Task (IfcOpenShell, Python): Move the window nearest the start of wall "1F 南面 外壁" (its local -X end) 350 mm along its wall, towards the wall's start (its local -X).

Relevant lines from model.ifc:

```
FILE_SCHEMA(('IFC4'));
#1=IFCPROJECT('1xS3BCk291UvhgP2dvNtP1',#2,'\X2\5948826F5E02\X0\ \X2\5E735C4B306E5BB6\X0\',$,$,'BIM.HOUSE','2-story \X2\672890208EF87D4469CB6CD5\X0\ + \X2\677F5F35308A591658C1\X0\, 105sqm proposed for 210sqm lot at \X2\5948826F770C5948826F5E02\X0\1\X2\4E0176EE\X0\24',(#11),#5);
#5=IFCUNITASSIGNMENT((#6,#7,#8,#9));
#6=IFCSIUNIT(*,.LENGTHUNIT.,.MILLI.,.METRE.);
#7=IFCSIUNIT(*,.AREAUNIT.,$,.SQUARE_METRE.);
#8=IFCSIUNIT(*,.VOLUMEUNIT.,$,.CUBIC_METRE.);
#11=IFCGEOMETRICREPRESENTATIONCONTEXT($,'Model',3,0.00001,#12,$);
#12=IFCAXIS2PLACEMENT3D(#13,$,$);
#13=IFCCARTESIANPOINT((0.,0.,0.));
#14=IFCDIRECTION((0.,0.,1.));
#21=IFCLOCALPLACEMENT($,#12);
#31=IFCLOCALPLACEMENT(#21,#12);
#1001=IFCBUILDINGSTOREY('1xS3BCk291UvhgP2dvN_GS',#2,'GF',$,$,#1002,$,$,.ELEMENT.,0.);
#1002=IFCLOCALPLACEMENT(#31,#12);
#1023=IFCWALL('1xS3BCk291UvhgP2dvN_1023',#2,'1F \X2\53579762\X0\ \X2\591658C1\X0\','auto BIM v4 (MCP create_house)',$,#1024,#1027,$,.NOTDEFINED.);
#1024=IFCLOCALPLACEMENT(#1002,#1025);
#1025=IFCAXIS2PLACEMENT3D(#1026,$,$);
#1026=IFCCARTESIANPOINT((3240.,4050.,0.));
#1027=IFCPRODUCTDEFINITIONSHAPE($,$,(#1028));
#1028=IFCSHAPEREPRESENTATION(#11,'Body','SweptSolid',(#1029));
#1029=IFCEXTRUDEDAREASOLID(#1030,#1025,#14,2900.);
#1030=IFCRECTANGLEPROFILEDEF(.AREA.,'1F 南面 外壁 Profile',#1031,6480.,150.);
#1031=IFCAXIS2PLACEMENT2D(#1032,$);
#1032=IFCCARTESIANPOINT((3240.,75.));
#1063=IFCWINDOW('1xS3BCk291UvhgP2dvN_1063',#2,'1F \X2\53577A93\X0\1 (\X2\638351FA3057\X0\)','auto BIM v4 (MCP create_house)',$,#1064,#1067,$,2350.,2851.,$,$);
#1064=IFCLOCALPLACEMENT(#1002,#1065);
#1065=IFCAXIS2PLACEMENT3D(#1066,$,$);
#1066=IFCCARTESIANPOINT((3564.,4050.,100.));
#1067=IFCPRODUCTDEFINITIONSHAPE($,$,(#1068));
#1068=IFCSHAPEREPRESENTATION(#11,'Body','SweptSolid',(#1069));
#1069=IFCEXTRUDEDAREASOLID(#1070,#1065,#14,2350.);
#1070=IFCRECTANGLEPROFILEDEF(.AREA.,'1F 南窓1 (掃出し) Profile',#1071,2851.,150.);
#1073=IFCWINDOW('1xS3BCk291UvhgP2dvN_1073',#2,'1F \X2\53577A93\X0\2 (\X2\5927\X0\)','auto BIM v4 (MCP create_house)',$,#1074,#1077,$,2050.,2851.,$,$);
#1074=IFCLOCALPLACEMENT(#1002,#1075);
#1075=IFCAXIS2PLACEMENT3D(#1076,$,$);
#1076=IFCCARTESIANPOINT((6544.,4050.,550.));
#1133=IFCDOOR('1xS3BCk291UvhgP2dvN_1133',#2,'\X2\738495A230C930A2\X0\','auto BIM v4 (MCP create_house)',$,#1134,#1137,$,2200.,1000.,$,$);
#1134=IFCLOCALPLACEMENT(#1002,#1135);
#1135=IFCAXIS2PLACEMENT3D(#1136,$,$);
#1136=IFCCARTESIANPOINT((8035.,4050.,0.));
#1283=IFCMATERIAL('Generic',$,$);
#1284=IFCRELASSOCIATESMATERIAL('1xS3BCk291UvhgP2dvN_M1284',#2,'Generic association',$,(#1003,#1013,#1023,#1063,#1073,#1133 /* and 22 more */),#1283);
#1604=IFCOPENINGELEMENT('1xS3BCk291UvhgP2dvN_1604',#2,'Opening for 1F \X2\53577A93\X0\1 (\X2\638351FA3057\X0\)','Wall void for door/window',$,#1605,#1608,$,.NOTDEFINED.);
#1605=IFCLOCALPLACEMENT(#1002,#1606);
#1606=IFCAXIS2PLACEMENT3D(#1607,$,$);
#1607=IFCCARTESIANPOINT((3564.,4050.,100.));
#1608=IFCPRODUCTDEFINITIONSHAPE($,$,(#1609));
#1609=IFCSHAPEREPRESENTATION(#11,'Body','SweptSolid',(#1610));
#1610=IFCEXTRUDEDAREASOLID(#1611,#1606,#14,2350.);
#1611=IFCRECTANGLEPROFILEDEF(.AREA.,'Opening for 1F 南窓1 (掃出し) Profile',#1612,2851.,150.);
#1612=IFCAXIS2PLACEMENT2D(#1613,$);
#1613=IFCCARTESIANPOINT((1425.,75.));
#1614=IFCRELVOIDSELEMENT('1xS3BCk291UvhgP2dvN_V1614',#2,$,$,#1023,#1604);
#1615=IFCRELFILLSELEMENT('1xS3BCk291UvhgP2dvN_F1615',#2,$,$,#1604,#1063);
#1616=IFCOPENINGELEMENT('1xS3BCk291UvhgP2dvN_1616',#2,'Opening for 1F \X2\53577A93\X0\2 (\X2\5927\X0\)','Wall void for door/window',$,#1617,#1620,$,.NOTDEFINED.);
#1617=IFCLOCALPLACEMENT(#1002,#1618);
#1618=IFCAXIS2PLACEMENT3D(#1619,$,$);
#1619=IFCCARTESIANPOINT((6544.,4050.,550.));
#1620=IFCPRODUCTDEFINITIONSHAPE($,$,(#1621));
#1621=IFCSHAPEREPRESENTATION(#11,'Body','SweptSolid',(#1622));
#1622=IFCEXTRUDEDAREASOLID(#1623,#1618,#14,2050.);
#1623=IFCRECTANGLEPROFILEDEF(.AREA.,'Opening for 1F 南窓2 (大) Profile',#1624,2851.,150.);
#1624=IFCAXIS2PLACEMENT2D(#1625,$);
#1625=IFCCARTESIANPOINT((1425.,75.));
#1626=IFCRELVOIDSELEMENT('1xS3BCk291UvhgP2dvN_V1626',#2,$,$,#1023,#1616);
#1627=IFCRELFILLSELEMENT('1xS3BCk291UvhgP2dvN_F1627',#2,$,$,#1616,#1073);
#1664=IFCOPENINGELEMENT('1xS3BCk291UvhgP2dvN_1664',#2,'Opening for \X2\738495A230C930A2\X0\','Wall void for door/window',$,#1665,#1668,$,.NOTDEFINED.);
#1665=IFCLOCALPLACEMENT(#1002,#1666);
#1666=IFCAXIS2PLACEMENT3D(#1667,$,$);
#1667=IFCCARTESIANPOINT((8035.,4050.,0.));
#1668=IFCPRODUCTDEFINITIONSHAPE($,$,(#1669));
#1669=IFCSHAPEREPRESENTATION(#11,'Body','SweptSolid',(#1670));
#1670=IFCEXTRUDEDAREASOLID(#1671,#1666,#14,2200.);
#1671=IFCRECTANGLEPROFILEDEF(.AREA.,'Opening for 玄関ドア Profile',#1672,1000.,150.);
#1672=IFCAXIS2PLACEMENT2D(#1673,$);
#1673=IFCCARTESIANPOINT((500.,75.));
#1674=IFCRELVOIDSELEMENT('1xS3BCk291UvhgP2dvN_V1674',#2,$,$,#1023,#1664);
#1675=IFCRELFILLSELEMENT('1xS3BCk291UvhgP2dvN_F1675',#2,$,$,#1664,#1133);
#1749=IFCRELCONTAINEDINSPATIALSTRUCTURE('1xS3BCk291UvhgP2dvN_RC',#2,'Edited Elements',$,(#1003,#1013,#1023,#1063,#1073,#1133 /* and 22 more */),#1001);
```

```python
import ifcopenshell
import ifcopenshell.api.geometry
import ifcopenshell.util.placement
import ifcopenshell.util.unit

model = ifcopenshell.open("model.ifc")
unit_scale = ifcopenshell.util.unit.calculate_unit_scale(model)

window = model.by_guid("1xS3BCk291UvhgP2dvN_1063")
opening = window.FillsVoids[0].RelatingOpeningElement
wall = opening.VoidsElements[0].RelatingBuildingElement

wall_matrix = ifcopenshell.util.placement.get_local_placement(wall.ObjectPlacement)
shift = wall_matrix[:3, 0] * -0.35 / unit_scale
before = ifcopenshell.util.placement.get_local_placement(window.ObjectPlacement)[:3, 3].copy()

# The window is not placed relative to its opening, so move both.
for product in (opening, window):
    matrix = ifcopenshell.util.placement.get_local_placement(product.ObjectPlacement)
    matrix[:3, 3] += shift
    ifcopenshell.api.geometry.edit_object_placement(model, product=product, matrix=matrix, is_si=False)

after = ifcopenshell.util.placement.get_local_placement(window.ObjectPlacement)[:3, 3]
print("window moved by", (after - before).round(3) + 0.0)

model.write("model_edited.ifc")
```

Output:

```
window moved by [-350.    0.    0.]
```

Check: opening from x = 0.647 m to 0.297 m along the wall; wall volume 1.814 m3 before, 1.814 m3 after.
